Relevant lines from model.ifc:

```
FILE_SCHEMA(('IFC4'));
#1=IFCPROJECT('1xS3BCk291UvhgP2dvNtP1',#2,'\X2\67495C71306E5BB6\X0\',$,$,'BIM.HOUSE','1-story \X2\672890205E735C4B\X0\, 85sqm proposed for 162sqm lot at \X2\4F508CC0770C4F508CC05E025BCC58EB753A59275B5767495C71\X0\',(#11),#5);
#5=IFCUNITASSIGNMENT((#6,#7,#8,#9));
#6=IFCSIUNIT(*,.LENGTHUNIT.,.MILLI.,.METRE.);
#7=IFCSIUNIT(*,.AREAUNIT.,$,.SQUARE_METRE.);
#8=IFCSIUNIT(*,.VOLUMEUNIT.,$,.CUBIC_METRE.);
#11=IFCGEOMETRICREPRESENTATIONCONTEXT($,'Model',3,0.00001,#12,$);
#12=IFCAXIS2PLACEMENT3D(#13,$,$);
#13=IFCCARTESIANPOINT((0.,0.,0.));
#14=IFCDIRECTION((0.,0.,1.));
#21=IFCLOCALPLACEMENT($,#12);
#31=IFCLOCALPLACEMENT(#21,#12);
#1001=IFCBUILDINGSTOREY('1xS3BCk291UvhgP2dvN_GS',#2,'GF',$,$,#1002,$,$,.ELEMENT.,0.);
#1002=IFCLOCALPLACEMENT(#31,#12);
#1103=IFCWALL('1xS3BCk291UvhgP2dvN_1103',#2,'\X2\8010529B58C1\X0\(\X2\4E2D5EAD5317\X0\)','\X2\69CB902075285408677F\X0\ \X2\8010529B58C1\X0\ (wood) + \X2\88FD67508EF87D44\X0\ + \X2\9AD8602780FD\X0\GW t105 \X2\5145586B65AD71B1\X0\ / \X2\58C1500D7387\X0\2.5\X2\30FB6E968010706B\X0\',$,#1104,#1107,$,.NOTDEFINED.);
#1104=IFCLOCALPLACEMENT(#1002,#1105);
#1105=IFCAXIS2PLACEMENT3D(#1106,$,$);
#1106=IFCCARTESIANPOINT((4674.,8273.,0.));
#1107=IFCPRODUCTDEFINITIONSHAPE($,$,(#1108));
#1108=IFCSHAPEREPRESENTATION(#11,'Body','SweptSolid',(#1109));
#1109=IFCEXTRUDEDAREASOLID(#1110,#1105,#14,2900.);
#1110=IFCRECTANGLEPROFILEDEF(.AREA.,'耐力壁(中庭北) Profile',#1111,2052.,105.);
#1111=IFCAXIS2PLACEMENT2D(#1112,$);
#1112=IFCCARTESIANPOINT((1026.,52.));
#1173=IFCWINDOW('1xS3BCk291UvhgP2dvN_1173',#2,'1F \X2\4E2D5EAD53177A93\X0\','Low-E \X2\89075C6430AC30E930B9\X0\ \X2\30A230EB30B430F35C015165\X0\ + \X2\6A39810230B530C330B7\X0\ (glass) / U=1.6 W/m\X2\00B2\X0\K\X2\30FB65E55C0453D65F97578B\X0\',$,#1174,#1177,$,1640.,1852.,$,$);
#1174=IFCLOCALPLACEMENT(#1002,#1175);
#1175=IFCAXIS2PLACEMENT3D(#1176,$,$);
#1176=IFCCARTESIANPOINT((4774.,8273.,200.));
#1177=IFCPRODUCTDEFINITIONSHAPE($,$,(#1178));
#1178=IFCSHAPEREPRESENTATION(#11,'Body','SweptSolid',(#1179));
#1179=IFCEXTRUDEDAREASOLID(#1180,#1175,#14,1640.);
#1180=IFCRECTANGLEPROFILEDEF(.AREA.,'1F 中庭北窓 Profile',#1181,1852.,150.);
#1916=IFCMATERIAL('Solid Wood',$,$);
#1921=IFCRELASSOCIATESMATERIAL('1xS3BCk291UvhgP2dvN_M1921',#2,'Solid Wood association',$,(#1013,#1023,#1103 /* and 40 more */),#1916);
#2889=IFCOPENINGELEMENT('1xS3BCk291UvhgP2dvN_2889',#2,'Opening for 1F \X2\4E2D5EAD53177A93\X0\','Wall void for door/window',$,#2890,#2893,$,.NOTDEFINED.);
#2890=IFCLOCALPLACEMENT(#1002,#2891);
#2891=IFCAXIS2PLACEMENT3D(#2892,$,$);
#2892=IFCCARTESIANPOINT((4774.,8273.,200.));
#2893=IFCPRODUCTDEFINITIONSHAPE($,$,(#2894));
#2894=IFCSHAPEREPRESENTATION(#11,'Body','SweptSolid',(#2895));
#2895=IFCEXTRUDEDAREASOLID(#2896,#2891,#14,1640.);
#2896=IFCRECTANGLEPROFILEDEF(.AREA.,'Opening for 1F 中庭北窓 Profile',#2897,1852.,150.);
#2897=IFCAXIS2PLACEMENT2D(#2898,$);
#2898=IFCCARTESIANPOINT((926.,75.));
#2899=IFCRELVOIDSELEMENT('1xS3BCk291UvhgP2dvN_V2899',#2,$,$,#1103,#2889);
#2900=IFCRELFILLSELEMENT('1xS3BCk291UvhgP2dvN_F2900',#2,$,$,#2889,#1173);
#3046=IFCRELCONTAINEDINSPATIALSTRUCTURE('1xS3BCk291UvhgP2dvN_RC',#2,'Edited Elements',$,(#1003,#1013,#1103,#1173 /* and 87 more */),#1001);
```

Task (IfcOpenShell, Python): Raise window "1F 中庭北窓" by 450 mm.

```python
import numpy as np
import ifcopenshell
import ifcopenshell.api.geometry
import ifcopenshell.util.placement
import ifcopenshell.util.unit

model = ifcopenshell.open("model.ifc")
unit_scale = ifcopenshell.util.unit.calculate_unit_scale(model)

window = model.by_guid("1xS3BCk291UvhgP2dvN_1173")
opening = window.FillsVoids[0].RelatingOpeningElement
dz = 0.45 / unit_scale

shift = np.array([0.0, 0.0, dz])
# The window is not placed relative to its opening, so move both.
for product in (opening, window):
    matrix = ifcopenshell.util.placement.get_local_placement(product.ObjectPlacement)
    matrix[:3, 3] += shift
    ifcopenshell.api.geometry.edit_object_placement(model, product=product, matrix=matrix, is_si=False)

print(f"moved by {dz * unit_scale:+.3f} m")

model.write("model_edited.ifc")
```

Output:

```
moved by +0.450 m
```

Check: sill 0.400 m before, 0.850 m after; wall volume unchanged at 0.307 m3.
